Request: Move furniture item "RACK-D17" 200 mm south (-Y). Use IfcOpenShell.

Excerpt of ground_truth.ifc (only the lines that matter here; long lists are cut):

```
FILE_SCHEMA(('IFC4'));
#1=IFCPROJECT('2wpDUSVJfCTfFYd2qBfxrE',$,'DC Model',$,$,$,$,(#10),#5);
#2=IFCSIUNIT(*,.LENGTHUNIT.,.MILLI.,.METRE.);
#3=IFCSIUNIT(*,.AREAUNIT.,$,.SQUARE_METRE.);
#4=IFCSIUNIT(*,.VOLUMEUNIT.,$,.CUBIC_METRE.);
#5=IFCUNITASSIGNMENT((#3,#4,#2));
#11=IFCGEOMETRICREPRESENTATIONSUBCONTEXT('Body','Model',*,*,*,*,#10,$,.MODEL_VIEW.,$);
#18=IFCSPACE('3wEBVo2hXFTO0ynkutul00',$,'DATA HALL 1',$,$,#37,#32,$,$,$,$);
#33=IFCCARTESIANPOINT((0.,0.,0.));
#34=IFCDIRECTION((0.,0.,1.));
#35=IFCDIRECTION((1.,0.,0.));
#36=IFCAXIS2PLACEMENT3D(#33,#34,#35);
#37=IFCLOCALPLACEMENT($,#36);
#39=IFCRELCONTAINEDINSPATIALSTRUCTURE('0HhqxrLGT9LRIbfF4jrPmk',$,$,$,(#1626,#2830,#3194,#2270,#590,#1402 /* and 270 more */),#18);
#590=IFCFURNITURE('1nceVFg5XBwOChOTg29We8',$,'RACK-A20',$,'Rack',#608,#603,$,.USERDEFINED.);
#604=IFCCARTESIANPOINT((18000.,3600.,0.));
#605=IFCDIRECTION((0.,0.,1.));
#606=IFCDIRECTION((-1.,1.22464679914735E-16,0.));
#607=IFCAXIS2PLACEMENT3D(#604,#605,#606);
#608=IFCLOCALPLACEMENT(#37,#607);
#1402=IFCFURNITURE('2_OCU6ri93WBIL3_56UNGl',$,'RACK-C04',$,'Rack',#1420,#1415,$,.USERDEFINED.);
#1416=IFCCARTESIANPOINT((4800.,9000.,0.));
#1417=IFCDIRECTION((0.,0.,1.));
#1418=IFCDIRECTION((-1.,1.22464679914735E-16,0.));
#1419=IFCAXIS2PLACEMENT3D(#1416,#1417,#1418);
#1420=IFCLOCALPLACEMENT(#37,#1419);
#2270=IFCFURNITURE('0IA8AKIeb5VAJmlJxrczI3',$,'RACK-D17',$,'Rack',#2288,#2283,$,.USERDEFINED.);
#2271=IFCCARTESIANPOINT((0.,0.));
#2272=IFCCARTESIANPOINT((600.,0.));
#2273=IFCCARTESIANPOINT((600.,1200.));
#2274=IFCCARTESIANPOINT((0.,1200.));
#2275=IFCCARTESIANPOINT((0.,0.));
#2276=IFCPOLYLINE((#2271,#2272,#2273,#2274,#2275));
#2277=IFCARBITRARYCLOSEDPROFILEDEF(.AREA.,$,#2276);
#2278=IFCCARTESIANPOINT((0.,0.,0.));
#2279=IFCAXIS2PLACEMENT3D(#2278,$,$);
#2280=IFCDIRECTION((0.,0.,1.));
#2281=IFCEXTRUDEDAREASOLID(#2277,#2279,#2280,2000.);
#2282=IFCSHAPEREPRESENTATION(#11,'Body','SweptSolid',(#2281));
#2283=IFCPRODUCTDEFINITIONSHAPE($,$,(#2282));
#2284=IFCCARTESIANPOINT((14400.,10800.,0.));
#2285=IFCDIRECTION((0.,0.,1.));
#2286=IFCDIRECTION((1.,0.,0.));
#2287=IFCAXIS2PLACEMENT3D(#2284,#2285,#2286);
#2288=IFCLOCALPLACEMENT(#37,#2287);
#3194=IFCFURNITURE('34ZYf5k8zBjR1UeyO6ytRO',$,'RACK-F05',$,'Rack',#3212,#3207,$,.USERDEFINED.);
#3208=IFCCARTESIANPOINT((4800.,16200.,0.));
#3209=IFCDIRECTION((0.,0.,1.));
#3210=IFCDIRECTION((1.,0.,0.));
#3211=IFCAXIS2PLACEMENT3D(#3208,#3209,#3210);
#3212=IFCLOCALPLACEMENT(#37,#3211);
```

```python
import ifcopenshell
import ifcopenshell.api.geometry
import ifcopenshell.util.placement

model = ifcopenshell.open("ground_truth.ifc")

item = model.by_id(2270)
matrix = ifcopenshell.util.placement.get_local_placement(item.ObjectPlacement)
matrix[1, 3] -= 200.0
ifcopenshell.api.geometry.edit_object_placement(model, product=item, matrix=matrix, is_si=False)

print(ifcopenshell.util.placement.get_local_placement(item.ObjectPlacement).round(3) + 0.0)

model.write("ground_truth_updated.ifc")
```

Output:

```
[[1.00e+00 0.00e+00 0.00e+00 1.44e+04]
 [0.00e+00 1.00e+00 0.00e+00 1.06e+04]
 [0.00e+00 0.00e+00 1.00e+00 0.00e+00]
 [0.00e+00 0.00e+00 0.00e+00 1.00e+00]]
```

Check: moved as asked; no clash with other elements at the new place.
